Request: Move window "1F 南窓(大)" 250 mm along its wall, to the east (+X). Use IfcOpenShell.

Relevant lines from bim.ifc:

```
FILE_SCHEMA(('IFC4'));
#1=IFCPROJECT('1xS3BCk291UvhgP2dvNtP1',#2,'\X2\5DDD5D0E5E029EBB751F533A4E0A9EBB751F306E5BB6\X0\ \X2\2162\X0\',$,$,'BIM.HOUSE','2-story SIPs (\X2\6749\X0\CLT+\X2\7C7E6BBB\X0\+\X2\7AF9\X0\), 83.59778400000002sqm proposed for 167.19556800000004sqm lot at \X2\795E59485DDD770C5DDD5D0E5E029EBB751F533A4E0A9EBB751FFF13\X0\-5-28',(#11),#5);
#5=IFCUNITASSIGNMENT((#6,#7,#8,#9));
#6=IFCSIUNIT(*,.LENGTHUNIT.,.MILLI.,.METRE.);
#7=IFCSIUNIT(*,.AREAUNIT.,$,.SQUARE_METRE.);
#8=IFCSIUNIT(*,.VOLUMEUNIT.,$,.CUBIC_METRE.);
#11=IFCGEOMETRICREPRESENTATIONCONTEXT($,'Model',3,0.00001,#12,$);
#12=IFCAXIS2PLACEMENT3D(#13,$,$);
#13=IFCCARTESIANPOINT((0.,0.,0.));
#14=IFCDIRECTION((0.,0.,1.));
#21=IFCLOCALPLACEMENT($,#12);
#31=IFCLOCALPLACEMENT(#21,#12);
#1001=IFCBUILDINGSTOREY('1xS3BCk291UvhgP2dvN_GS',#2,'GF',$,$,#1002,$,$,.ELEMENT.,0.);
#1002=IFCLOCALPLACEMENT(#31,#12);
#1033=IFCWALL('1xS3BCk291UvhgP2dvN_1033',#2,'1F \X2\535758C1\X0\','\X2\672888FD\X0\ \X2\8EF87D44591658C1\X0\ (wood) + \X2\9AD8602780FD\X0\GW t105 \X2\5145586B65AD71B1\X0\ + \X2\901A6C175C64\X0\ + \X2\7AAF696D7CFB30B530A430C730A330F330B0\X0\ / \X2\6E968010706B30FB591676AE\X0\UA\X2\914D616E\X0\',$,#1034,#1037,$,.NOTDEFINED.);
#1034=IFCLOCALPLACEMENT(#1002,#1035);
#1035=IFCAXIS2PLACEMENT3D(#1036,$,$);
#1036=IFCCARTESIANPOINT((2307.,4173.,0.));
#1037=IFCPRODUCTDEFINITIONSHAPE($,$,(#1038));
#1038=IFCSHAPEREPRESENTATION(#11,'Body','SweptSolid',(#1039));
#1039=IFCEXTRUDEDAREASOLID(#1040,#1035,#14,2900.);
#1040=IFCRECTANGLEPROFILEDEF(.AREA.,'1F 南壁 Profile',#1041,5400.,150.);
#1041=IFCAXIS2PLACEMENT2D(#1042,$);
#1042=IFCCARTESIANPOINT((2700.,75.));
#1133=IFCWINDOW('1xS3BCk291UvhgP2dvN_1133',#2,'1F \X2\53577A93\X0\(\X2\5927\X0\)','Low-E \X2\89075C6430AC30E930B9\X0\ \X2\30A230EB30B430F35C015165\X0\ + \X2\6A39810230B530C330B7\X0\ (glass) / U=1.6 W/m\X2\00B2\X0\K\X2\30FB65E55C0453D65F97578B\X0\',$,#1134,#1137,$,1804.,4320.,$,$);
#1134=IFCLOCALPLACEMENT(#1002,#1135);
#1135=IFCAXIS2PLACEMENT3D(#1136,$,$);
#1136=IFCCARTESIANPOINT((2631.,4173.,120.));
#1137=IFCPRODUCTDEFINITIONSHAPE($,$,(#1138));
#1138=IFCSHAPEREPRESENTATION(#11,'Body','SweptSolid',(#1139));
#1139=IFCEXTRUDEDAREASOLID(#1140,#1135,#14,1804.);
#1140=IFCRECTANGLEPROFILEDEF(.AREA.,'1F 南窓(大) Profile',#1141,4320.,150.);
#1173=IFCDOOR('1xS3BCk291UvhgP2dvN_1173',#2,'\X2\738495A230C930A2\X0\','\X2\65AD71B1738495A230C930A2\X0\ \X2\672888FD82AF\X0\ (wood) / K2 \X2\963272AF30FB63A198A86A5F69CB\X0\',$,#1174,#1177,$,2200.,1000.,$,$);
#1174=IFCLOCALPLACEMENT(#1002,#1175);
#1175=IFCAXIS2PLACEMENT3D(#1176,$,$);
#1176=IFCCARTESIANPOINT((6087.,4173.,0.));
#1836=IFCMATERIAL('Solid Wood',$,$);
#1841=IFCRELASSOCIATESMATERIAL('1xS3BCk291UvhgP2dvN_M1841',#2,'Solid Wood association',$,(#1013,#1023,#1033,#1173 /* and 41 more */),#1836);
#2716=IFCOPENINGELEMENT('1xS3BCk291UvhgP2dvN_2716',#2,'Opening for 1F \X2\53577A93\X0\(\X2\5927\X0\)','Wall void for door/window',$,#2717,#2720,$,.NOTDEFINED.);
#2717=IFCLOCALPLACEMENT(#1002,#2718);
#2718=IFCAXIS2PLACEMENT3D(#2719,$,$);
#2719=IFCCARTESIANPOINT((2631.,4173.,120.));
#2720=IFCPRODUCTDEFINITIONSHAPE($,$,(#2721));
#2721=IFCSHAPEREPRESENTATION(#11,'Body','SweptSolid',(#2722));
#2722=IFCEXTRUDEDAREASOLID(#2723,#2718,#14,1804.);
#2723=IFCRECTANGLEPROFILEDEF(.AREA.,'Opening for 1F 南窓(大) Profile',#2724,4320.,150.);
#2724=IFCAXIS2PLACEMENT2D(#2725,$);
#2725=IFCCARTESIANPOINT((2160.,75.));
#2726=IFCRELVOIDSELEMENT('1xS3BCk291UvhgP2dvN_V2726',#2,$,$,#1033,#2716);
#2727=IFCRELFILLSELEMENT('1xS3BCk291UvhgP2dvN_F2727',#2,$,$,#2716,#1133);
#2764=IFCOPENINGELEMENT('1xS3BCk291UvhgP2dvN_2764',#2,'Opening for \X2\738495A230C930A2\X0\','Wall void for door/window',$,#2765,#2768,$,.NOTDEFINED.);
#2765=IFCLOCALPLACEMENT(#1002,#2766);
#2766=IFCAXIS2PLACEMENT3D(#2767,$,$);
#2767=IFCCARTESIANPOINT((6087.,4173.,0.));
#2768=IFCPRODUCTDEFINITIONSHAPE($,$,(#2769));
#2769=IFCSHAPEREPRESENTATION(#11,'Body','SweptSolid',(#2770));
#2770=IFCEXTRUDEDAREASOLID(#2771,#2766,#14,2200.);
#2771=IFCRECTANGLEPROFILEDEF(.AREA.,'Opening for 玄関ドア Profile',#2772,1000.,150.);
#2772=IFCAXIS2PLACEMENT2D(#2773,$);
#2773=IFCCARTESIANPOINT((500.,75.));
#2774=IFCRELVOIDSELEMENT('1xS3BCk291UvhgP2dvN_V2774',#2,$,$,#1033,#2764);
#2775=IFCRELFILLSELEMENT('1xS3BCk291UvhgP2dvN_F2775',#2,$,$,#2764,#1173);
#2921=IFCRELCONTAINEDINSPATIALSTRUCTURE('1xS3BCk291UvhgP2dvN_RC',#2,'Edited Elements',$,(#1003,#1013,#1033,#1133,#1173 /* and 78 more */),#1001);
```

```python
import ifcopenshell
import ifcopenshell.api.geometry
import ifcopenshell.util.placement
import ifcopenshell.util.unit

model = ifcopenshell.open("bim.ifc")
unit_scale = ifcopenshell.util.unit.calculate_unit_scale(model)

window = model.by_id(1133)
opening = window.FillsVoids[0].RelatingOpeningElement
wall = opening.VoidsElements[0].RelatingBuildingElement

wall_matrix = ifcopenshell.util.placement.get_local_placement(wall.ObjectPlacement)
shift = wall_matrix[:3, 0] * 0.25 / unit_scale
before = ifcopenshell.util.placement.get_local_placement(window.ObjectPlacement)[:3, 3].copy()

# The window is not placed relative to its opening, so move both.
for product in (opening, window):
    matrix = ifcopenshell.util.placement.get_local_placement(product.ObjectPlacement)
    matrix[:3, 3] += shift
    ifcopenshell.api.geometry.edit_object_placement(model, product=product, matrix=matrix, is_si=False)

after = ifcopenshell.util.placement.get_local_placement(window.ObjectPlacement)[:3, 3]
print("window moved by", (after - before).round(3) + 0.0)

model.write("bim_edited.ifc")
```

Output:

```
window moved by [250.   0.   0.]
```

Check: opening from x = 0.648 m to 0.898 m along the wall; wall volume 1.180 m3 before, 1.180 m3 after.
